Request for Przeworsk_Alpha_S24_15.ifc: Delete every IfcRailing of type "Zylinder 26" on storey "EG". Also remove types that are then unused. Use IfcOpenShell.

First a look at what the model holds.

```python
import ifcopenshell
import ifcopenshell.util.element

model = ifcopenshell.open("Przeworsk_Alpha_S24_15.ifc")
print(model.schema)
storey = next(s for s in model.by_type("IfcBuildingStorey") if s.Name == "EG")
railings = [e for e in ifcopenshell.util.element.get_decomposition(storey) if e.is_a("IfcRailing")]
seen = {}
for e in railings:
    element_type = ifcopenshell.util.element.get_type(e)
    name = element_type.Name if element_type not in (None, e) else None
    seen[name] = seen.get(name, 0) + 1
for name, count in sorted(seen.items(), key=str):
    print(count, "x", name)
```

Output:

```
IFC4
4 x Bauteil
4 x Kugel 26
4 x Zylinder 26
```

```python
import ifcopenshell
import ifcopenshell.api.root
import ifcopenshell.util.element

model = ifcopenshell.open("Przeworsk_Alpha_S24_15.ifc")

storey = next(s for s in model.by_type("IfcBuildingStorey") if s.Name == "EG")
railings = [e for e in ifcopenshell.util.element.get_decomposition(storey) if e.is_a("IfcRailing")]
targets = [e for e in railings if (t := ifcopenshell.util.element.get_type(e)) not in (None, e) and t.Name == "Zylinder 26"]
types = {ifcopenshell.util.element.get_type(e) for e in targets} - {None, *targets}

for e in targets:
    ifcopenshell.api.root.remove_product(model, product=e)
print(len(targets), "removed")

unused = [t for t in types if not ifcopenshell.util.element.get_types(t)]
for t in unused:
    ifcopenshell.api.root.remove_product(model, product=t)
print(len(unused), "unused types removed")

model.write("Przeworsk_Alpha_S24_15_updated.ifc")
```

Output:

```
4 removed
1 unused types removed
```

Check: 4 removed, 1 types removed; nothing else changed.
